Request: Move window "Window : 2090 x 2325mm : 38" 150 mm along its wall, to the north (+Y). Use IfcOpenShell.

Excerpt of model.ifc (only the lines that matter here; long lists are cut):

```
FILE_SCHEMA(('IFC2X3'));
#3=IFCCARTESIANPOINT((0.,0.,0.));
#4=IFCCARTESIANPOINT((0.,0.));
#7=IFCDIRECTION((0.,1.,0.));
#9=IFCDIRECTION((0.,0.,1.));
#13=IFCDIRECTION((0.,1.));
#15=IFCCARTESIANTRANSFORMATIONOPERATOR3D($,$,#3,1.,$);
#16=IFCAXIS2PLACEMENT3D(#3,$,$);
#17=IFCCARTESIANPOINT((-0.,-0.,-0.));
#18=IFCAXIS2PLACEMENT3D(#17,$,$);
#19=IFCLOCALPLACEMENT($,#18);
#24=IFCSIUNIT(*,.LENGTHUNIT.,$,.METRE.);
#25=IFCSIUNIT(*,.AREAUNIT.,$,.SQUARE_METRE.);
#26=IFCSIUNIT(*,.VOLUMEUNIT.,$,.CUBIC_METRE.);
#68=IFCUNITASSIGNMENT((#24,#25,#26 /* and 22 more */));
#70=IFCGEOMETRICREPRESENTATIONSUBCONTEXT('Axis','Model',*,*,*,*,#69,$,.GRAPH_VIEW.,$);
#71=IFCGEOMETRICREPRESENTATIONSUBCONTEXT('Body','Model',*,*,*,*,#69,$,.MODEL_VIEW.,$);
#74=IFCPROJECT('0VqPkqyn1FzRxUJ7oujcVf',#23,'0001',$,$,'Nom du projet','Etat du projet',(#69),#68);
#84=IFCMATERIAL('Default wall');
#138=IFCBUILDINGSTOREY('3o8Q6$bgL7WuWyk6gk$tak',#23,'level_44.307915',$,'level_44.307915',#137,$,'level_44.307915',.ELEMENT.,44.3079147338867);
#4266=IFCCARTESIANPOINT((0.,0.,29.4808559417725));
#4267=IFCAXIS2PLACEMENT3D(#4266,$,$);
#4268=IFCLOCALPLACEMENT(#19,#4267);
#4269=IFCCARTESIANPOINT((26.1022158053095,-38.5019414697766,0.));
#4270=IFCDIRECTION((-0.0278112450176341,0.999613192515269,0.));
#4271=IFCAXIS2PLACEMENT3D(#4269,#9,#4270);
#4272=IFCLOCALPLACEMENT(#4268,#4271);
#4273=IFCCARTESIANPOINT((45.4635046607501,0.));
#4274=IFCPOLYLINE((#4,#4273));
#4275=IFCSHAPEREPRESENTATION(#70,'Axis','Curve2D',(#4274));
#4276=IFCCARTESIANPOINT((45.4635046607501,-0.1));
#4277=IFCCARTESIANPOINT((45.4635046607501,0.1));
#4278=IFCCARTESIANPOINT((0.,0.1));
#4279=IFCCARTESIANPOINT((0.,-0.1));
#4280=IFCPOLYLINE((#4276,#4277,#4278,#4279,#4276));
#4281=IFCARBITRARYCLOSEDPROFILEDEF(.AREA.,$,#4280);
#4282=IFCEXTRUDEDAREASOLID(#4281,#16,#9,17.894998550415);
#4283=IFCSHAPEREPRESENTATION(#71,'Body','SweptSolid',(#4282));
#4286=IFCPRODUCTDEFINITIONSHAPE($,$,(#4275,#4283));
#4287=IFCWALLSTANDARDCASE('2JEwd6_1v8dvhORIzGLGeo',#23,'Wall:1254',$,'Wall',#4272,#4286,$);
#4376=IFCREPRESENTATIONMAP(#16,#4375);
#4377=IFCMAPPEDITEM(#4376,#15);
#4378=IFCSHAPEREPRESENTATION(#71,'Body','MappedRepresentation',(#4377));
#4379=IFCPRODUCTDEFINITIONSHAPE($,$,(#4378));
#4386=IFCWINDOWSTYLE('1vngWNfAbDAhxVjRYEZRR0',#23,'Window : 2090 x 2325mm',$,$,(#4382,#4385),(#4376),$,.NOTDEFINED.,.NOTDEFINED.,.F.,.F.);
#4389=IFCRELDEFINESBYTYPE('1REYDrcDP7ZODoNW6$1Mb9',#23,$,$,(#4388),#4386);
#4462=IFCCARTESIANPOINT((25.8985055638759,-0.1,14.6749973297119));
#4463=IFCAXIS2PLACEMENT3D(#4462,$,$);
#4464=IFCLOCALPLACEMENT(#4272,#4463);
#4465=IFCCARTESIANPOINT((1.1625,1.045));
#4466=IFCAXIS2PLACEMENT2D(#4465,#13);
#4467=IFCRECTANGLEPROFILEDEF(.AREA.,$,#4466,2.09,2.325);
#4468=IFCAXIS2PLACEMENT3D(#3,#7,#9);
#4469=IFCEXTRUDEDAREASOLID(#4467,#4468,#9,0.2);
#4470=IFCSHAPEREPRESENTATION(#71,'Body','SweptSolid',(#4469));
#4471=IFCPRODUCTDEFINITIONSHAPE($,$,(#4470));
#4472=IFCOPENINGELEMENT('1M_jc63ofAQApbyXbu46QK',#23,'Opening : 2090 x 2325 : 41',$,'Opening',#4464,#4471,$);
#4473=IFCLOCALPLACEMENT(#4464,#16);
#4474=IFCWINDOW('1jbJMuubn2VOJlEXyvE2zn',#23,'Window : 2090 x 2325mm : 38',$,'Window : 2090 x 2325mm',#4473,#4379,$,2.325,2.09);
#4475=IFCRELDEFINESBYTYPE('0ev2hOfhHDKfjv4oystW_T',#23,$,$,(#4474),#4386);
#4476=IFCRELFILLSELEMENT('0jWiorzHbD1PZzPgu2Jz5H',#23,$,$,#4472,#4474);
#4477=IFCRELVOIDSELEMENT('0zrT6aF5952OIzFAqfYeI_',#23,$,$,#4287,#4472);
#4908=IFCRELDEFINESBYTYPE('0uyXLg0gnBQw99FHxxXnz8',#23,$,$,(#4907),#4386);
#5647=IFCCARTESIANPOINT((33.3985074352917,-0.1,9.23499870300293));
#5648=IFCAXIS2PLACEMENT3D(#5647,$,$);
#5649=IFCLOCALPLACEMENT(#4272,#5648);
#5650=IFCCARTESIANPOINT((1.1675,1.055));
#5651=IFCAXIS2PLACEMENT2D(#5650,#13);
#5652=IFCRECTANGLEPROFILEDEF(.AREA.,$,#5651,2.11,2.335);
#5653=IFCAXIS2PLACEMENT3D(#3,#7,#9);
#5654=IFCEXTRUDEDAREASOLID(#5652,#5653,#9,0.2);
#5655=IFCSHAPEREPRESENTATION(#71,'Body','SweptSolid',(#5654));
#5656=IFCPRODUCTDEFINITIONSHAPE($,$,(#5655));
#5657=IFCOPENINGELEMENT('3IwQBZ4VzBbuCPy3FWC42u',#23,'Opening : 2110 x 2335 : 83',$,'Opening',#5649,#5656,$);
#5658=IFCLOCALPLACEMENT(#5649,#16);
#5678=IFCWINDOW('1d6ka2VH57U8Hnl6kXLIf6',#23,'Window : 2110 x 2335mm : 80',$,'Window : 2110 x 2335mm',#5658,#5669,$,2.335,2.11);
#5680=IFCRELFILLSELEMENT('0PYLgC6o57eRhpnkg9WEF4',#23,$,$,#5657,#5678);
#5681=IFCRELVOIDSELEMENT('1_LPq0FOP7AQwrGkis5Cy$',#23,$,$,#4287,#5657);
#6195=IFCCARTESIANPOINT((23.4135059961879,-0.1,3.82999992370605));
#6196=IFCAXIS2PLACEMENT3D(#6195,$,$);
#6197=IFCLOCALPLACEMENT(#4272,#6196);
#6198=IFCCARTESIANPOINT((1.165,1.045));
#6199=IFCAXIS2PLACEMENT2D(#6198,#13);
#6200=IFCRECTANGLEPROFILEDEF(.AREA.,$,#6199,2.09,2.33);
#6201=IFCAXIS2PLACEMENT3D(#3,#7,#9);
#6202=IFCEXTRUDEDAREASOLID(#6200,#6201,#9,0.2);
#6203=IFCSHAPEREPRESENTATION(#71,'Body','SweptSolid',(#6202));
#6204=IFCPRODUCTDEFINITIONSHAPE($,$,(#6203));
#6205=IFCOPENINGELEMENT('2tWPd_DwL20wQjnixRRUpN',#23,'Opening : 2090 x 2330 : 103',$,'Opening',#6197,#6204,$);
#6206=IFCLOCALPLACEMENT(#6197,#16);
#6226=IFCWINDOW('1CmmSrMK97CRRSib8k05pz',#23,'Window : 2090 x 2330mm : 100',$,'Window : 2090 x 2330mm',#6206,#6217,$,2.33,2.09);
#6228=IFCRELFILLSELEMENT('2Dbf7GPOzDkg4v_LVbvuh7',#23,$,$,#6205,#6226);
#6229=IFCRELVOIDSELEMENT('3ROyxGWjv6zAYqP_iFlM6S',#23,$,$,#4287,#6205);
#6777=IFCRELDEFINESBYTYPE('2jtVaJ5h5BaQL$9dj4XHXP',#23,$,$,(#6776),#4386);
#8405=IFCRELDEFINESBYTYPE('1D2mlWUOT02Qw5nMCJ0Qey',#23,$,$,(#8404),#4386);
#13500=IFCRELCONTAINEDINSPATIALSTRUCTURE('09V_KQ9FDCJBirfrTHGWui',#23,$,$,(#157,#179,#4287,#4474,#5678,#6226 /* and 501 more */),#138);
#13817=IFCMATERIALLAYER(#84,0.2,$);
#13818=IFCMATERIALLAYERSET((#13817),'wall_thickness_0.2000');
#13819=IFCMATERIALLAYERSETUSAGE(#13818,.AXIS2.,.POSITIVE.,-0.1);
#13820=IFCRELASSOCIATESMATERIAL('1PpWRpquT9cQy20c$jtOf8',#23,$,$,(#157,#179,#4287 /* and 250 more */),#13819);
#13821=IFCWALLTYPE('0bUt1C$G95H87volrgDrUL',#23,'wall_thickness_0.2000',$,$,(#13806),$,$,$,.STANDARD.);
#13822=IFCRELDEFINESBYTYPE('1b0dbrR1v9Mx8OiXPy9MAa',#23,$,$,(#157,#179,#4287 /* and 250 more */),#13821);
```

```python
import ifcopenshell
import ifcopenshell.api.geometry
import ifcopenshell.util.placement

model = ifcopenshell.open("model.ifc")

window = model.by_id(4474)
opening = window.FillsVoids[0].RelatingOpeningElement
wall = opening.VoidsElements[0].RelatingBuildingElement

wall_matrix = ifcopenshell.util.placement.get_local_placement(wall.ObjectPlacement)
shift = wall_matrix[:3, 0] * 0.15
before = ifcopenshell.util.placement.get_local_placement(window.ObjectPlacement)[:3, 3].copy()

# The window is placed relative to its opening, so it follows when the opening moves.
matrix = ifcopenshell.util.placement.get_local_placement(opening.ObjectPlacement)
matrix[:3, 3] += shift
ifcopenshell.api.geometry.edit_object_placement(
    model, product=opening, matrix=matrix, is_si=False, should_transform_children=True
)

after = ifcopenshell.util.placement.get_local_placement(window.ObjectPlacement)[:3, 3]
print("window moved by", (after - before).round(3) + 0.0)

model.write("model-out.ifc")
```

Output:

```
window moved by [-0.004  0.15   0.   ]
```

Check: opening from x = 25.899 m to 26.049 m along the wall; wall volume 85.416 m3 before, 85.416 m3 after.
